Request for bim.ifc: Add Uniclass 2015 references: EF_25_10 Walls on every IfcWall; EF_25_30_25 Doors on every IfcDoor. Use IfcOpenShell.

First a look at what the model holds.

```python
import ifcopenshell

model = ifcopenshell.open("bim.ifc")
print(model.schema)
print("classifications:", [c.Name for c in model.by_type("IfcClassification")])
for ifc_class in ("IfcDoor", "IfcRoof", "IfcStair", "IfcWall", "IfcWindow"):
    print(ifc_class, len(model.by_type(ifc_class)))
```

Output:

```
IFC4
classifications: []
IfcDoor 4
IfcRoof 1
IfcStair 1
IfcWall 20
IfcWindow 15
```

```python
import ifcopenshell
import ifcopenshell.api.classification

model = ifcopenshell.open("bim.ifc")

system = ifcopenshell.api.classification.add_classification(model, classification="Uniclass 2015")

codes = {
    "IfcWall": ("EF_25_10", "Walls"),
    "IfcDoor": ("EF_25_30_25", "Doors"),
}
for ifc_class, (code, name) in codes.items():
    products = model.by_type(ifc_class)
    ifcopenshell.api.classification.add_reference(
        model, products=products, classification=system, identification=code, name=name
    )
    print(code, len(products))

model.write("bim_v2.ifc")
```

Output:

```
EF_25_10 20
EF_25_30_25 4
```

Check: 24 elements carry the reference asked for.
